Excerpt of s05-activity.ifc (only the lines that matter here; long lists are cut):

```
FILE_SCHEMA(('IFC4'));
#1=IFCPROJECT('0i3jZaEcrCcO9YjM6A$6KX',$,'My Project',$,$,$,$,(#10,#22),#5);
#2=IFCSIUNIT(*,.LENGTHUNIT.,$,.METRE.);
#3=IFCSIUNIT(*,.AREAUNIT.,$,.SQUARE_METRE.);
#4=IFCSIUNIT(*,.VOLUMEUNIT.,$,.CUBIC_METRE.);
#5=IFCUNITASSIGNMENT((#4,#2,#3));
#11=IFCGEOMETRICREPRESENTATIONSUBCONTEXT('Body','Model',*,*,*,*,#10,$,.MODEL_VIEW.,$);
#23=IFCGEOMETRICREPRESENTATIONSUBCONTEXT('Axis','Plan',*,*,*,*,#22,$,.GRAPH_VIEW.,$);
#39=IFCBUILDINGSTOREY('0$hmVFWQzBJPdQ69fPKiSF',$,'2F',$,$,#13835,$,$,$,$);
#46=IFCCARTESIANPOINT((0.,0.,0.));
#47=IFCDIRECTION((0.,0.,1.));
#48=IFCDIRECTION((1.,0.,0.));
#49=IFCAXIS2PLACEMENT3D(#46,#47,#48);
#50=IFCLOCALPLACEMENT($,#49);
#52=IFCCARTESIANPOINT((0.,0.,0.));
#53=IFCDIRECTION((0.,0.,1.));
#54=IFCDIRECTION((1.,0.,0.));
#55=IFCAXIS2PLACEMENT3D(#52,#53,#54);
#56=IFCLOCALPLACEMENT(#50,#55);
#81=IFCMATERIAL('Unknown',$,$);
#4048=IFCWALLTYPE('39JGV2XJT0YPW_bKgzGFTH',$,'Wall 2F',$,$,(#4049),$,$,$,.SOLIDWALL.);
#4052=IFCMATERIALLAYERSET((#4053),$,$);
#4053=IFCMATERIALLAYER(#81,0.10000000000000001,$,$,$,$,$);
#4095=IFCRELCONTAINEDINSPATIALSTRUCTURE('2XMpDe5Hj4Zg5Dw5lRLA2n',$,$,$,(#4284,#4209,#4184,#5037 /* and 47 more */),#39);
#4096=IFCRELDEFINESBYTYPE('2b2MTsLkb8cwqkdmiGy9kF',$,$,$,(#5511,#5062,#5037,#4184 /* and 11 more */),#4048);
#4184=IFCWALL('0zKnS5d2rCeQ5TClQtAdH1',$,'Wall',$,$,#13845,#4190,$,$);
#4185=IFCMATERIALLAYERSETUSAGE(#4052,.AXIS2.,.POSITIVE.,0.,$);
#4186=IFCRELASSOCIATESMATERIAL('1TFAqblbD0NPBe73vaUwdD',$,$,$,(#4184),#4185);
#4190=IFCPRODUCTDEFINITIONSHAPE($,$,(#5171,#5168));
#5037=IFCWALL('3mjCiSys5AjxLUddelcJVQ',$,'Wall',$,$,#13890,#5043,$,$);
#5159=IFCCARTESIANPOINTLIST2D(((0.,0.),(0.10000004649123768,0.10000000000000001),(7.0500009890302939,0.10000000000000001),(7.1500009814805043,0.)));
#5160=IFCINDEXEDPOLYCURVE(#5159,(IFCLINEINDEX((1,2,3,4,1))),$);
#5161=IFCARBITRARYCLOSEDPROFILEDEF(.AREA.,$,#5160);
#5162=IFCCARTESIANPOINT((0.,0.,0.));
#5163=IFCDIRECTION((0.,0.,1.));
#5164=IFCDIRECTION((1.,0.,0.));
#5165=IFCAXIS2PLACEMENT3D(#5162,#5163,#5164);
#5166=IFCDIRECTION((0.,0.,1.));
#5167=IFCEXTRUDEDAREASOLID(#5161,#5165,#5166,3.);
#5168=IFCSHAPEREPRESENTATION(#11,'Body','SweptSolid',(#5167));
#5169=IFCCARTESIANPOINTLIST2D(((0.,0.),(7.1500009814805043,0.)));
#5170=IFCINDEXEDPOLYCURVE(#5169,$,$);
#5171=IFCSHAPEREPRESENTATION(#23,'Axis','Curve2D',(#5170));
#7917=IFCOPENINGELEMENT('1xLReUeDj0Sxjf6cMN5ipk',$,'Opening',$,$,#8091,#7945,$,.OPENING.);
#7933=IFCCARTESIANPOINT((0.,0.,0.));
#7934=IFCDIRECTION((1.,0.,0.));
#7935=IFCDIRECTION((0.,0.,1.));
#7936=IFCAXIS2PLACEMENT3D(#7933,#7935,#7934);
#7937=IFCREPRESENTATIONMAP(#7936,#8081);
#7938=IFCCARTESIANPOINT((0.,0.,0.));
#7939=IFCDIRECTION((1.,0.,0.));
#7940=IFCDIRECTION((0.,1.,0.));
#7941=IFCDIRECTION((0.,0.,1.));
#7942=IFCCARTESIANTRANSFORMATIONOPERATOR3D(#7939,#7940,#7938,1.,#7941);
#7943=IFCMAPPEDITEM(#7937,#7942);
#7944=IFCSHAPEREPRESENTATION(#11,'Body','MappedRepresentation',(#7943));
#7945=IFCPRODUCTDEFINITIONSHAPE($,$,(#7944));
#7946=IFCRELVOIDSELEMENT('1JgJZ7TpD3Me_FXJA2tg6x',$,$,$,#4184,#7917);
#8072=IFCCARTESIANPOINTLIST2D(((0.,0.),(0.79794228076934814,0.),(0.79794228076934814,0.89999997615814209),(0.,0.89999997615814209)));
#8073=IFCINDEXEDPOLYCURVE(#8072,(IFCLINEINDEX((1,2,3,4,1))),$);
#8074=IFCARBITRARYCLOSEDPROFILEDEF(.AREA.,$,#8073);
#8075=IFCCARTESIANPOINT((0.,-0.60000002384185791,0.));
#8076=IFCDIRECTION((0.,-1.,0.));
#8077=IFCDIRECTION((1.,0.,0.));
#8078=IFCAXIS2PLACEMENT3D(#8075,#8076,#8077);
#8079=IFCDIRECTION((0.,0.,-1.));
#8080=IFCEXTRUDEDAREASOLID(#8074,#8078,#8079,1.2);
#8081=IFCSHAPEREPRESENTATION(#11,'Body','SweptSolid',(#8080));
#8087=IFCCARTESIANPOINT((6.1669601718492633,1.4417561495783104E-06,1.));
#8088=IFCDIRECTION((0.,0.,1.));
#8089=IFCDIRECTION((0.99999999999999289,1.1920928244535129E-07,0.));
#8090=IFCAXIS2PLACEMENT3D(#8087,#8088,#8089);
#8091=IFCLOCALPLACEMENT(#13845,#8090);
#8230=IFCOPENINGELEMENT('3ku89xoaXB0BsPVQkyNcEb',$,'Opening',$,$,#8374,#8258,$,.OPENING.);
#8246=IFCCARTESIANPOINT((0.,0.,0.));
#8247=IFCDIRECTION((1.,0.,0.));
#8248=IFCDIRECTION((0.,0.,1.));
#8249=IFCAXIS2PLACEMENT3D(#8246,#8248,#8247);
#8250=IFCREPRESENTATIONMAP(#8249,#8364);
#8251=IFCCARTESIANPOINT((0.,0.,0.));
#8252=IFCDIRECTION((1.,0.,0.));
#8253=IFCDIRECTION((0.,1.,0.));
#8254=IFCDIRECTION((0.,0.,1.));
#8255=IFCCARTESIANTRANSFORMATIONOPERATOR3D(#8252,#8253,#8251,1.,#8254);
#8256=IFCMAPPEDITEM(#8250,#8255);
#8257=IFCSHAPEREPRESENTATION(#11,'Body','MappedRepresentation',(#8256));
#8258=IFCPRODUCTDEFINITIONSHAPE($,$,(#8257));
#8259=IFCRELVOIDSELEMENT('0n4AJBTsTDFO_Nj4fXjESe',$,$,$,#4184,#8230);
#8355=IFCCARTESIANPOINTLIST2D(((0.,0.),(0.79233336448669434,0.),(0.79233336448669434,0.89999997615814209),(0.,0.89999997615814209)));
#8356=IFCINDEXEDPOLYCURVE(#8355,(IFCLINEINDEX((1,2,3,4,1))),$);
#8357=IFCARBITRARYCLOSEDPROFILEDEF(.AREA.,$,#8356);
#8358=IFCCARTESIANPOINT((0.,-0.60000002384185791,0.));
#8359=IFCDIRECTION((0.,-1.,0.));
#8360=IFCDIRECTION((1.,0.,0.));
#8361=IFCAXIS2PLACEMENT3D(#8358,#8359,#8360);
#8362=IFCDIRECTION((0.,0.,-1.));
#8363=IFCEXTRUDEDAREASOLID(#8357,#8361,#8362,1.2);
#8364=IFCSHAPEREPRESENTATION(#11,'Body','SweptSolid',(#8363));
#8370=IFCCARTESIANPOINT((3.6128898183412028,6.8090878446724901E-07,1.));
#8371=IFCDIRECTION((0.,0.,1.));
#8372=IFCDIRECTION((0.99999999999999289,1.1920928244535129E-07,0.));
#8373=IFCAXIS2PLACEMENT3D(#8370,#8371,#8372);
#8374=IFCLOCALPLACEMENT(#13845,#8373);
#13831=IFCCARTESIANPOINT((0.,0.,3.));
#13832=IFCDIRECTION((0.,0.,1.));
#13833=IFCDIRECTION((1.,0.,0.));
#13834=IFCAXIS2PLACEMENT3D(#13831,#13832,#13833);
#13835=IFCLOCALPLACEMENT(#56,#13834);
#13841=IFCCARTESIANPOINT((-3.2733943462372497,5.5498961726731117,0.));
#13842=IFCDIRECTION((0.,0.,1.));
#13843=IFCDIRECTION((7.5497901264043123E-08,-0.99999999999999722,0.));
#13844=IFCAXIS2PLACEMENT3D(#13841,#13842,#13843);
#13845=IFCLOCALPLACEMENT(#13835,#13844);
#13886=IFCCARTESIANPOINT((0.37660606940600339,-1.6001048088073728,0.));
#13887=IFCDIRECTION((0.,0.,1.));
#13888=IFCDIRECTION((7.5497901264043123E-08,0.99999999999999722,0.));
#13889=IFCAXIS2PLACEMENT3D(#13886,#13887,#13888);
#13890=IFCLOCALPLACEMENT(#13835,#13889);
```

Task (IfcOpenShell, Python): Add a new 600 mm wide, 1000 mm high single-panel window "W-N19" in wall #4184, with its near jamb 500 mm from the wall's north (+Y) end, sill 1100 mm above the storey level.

```python
import numpy as np
import ifcopenshell
import ifcopenshell.api.feature
import ifcopenshell.api.geometry
import ifcopenshell.api.root
import ifcopenshell.api.spatial
import ifcopenshell.geom
import ifcopenshell.util.element
import ifcopenshell.util.placement
import ifcopenshell.util.representation
import ifcopenshell.util.shape
import ifcopenshell.util.unit

model = ifcopenshell.open("s05-activity.ifc")
unit_scale = ifcopenshell.util.unit.calculate_unit_scale(model)
settings = ifcopenshell.geom.settings()


def volume(element):
    """Net volume in cubic metres, openings subtracted."""
    shape = ifcopenshell.geom.create_shape(settings, element)
    return ifcopenshell.util.shape.get_volume(shape.geometry)


wall = model.by_id(4184)
storey = ifcopenshell.util.element.get_container(wall, ifc_class="IfcBuildingStorey")
context = ifcopenshell.util.representation.get_context(model, "Model", "Body", "MODEL_VIEW")
before = volume(wall)

width, height, from_end, sill = 0.6, 1, 0.5, 1.1  # metres

# The wall runs along its own X axis, and the end named is its -X end.
wall_shape = ifcopenshell.geom.create_shape(settings, wall)
x, y, z = ifcopenshell.util.shape.get_vertices(wall_shape.geometry).T
start = x.min() + from_end
face, thickness = float(y.min()), float(y.max() - y.min())
wall_matrix = ifcopenshell.util.placement.get_local_placement(wall.ObjectPlacement)
level = ifcopenshell.util.placement.get_local_placement(storey.ObjectPlacement)[2, 3]


def in_wall(x, y):
    """Placement at x, y metres in the wall's axes, at sill height."""
    matrix = wall_matrix.copy()
    matrix[:, 3] = wall_matrix @ np.array([x / unit_scale, y / unit_scale, 0.0, 1.0])
    matrix[2, 3] = level + sill / unit_scale
    return matrix


# Opening: a box that overshoots both wall faces by 50 mm.
opening = ifcopenshell.api.root.create_entity(model, ifc_class="IfcOpeningElement", predefined_type="OPENING")
box = ifcopenshell.api.geometry.add_wall_representation(
    model, context=context, length=width, height=height, thickness=thickness + 0.1
)
ifcopenshell.api.geometry.assign_representation(model, product=opening, representation=box)
ifcopenshell.api.geometry.edit_object_placement(model, product=opening, matrix=in_wall(start, face - 0.05), is_si=False)
ifcopenshell.api.feature.add_feature(model, feature=opening, element=wall)

window = ifcopenshell.api.root.create_entity(model, ifc_class="IfcWindow", name="W-N19", predefined_type="WINDOW")
window.OverallWidth, window.OverallHeight = width / unit_scale, height / unit_scale
window.PartitioningType = "SINGLE_PANEL"
body = ifcopenshell.api.geometry.add_window_representation(
    model,
    context=context,
    overall_width=window.OverallWidth,
    overall_height=window.OverallHeight,
    partition_type="SINGLE_PANEL",
)
ifcopenshell.api.geometry.assign_representation(model, product=window, representation=body)
ifcopenshell.api.spatial.assign_container(model, products=[window], relating_structure=storey)
ifcopenshell.api.feature.add_filling(model, opening=opening, element=window)

# Centre the window in the wall's thickness.
ifcopenshell.api.geometry.edit_object_placement(model, product=window, matrix=in_wall(start, face), is_si=False)
window_shape = ifcopenshell.geom.create_shape(settings, window)
depth = ifcopenshell.util.shape.get_vertices(window_shape.geometry)[:, 1]
offset = face + thickness / 2 - (depth.min() + depth.max()) / 2
ifcopenshell.api.geometry.edit_object_placement(model, product=window, matrix=in_wall(start, offset), is_si=False)

after = volume(wall)

print(f"wall volume {before:.3f} -> {after:.3f} m3")

model.write("s05-activity_v2.ifc")
```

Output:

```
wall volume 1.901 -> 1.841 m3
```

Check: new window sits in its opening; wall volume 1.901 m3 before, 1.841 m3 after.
